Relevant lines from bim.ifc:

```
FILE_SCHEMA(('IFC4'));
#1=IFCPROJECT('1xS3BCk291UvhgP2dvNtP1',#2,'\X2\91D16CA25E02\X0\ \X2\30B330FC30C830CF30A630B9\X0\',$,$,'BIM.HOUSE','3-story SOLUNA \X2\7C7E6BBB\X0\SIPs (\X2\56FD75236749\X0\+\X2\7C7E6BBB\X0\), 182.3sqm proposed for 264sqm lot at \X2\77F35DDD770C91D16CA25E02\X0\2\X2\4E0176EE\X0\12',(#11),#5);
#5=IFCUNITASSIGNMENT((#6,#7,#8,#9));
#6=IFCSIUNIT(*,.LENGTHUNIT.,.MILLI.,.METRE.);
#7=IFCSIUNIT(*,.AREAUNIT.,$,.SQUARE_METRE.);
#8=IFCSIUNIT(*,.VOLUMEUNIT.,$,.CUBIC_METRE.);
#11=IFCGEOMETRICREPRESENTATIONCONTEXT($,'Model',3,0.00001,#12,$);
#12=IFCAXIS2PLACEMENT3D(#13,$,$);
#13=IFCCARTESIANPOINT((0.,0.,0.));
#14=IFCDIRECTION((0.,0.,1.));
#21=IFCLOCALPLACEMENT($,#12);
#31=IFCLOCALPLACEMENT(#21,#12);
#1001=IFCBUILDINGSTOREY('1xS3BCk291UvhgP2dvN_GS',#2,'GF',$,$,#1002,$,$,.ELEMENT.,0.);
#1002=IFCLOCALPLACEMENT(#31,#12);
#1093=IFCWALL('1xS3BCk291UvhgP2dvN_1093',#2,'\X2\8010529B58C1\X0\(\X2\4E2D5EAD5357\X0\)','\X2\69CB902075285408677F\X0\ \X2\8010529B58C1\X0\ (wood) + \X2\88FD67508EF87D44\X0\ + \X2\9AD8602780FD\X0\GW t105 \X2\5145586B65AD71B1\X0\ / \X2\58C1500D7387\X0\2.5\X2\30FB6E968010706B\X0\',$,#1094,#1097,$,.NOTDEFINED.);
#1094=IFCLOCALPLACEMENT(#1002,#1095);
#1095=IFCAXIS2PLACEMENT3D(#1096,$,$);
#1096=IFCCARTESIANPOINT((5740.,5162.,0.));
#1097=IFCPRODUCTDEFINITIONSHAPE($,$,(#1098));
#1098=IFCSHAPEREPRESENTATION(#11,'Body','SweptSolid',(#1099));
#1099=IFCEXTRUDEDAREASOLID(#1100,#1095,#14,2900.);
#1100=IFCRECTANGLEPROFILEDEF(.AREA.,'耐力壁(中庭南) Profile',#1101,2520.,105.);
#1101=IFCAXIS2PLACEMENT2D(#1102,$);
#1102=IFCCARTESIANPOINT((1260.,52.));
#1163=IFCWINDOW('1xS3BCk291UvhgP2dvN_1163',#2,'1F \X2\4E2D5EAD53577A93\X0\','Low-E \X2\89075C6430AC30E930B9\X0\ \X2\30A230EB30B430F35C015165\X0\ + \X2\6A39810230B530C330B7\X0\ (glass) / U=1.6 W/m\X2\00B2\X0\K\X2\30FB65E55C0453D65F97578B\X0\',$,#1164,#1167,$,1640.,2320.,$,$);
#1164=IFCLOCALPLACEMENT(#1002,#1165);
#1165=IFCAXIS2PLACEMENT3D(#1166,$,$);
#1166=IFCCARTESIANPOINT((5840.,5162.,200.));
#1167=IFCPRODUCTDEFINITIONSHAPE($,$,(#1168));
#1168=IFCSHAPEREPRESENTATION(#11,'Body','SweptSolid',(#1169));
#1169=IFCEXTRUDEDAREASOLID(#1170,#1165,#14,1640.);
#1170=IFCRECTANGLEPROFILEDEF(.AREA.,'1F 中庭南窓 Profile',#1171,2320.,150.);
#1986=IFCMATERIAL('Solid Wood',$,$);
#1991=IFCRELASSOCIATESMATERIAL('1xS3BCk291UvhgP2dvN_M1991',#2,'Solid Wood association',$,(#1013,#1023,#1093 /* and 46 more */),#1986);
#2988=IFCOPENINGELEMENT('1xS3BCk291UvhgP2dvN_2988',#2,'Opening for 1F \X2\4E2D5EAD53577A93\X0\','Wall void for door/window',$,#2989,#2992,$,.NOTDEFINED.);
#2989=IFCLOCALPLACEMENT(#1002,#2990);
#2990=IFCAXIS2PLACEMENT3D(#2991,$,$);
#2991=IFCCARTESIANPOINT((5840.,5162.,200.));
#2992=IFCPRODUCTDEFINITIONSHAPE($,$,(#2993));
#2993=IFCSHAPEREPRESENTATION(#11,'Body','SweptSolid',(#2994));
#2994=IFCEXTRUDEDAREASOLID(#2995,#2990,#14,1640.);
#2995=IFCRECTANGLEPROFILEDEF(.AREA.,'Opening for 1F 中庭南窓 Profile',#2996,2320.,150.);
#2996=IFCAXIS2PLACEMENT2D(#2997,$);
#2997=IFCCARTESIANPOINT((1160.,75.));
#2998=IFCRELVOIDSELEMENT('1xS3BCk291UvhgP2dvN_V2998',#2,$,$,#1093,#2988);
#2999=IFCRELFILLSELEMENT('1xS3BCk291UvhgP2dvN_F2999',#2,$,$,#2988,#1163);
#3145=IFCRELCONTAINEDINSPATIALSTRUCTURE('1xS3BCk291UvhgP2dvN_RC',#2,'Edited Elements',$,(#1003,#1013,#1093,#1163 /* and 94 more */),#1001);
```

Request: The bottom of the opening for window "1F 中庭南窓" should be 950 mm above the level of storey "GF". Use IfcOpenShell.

```python
import numpy as np
import ifcopenshell
import ifcopenshell.api.geometry
import ifcopenshell.geom
import ifcopenshell.util.element
import ifcopenshell.util.placement
import ifcopenshell.util.shape
import ifcopenshell.util.unit

model = ifcopenshell.open("bim.ifc")
unit_scale = ifcopenshell.util.unit.calculate_unit_scale(model)

window = model.by_guid("1xS3BCk291UvhgP2dvN_1163")
opening = window.FillsVoids[0].RelatingOpeningElement
storey = ifcopenshell.util.element.get_container(window, ifc_class="IfcBuildingStorey")
level = ifcopenshell.util.placement.get_local_placement(storey.ObjectPlacement)[2, 3]

# The opening's origin need not be at the sill, so measure its lowest point.
shape = ifcopenshell.geom.create_shape(ifcopenshell.geom.settings(), opening)
bottom = ifcopenshell.util.shape.get_shape_bottom_elevation(shape, shape.geometry) / unit_scale
dz = level + 0.95 / unit_scale - bottom

shift = np.array([0.0, 0.0, dz])
# The window is not placed relative to its opening, so move both.
for product in (opening, window):
    matrix = ifcopenshell.util.placement.get_local_placement(product.ObjectPlacement)
    matrix[:3, 3] += shift
    ifcopenshell.api.geometry.edit_object_placement(model, product=product, matrix=matrix, is_si=False)

print(f"moved by {dz * unit_scale:+.3f} m")

model.write("bim_rev.ifc")
```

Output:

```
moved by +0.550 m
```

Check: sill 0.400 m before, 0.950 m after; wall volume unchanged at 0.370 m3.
